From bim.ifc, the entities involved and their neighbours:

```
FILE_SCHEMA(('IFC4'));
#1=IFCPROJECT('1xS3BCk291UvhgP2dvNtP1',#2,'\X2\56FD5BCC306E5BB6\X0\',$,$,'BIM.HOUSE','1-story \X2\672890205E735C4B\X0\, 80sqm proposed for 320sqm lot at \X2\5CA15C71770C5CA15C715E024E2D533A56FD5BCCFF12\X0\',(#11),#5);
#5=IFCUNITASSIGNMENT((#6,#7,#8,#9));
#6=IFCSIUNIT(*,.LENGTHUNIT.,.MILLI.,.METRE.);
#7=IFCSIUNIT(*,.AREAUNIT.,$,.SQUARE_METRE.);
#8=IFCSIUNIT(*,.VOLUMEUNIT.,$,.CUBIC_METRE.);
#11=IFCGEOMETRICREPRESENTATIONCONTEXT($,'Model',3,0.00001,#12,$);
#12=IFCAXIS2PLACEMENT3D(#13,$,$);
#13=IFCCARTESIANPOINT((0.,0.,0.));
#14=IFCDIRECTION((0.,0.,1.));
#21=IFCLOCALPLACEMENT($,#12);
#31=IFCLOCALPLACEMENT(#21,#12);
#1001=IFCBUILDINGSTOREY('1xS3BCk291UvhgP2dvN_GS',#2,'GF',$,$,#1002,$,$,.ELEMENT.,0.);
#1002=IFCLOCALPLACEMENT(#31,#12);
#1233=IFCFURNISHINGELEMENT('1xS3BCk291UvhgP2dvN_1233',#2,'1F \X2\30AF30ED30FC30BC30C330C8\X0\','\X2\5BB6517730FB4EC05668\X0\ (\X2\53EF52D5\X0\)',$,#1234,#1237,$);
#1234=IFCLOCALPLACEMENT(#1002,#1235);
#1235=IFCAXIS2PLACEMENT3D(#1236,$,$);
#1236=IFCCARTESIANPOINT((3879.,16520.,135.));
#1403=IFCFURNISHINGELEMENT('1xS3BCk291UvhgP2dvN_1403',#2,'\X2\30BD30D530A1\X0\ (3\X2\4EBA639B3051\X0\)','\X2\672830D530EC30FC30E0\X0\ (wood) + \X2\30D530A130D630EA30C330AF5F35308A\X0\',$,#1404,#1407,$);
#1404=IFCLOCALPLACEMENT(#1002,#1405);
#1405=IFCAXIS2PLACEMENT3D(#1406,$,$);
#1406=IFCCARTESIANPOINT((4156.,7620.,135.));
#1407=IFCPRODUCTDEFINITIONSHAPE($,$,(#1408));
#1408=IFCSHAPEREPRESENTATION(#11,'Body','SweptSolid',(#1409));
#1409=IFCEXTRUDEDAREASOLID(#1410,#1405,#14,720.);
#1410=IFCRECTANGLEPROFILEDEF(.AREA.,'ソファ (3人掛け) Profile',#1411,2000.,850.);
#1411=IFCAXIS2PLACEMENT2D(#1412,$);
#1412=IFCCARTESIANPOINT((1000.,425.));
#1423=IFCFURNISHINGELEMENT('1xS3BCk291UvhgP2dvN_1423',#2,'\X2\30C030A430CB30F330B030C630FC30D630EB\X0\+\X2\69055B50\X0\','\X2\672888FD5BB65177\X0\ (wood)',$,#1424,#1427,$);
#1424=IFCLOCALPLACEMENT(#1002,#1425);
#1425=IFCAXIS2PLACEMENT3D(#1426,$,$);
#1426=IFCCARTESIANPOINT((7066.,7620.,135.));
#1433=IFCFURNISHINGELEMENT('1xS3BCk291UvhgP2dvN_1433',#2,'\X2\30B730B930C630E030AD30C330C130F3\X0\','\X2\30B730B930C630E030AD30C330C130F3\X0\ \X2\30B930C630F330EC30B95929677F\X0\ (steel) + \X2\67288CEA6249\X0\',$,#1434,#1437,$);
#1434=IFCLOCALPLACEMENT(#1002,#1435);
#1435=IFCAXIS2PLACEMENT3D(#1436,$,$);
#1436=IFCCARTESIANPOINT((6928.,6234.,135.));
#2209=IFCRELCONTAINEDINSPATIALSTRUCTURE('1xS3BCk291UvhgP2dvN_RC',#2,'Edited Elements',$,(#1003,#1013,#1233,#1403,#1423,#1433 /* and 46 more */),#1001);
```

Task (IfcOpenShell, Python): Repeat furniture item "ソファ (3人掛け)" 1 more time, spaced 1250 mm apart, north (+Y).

```python
import numpy as np
import ifcopenshell
import ifcopenshell.api.geometry
import ifcopenshell.api.root
import ifcopenshell.util.element
import ifcopenshell.util.placement
import ifcopenshell.util.unit

model = ifcopenshell.open("bim.ifc")
unit_scale = ifcopenshell.util.unit.calculate_unit_scale(model)


def reuse_history(source, copy):
    """copy_class also copies each property set's owner history, people and application; keep the originals."""
    for rel in copy.IsDefinedBy:
        if rel.is_a("IfcRelDefinesByProperties") and (history := rel.RelatingPropertyDefinition.OwnerHistory):
            rel.RelatingPropertyDefinition.OwnerHistory = source.OwnerHistory
            ifcopenshell.util.element.remove_deep2(model, history)


source = model.by_guid("1xS3BCk291UvhgP2dvN_1403")
base = ifcopenshell.util.placement.get_local_placement(source.ObjectPlacement)
step = np.array([0.0, 1.0, 0.0]) * 1.25 / unit_scale

for i in range(1, 2):
    copy = ifcopenshell.api.root.copy_class(model, product=source)
    copy.Representation = ifcopenshell.util.element.copy_deep(
        model, source.Representation, exclude=["IfcGeometricRepresentationContext", "IfcRepresentationMap"]
    )
    reuse_history(source, copy)
    matrix = base.copy()
    matrix[:3, 3] += i * step
    print("added at", matrix[:3, 3].round(3) + 0.0)
    ifcopenshell.api.geometry.edit_object_placement(model, product=copy, matrix=matrix, is_si=False)

model.write("bim_v2.ifc")
```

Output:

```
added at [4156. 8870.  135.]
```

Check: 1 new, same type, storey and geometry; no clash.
